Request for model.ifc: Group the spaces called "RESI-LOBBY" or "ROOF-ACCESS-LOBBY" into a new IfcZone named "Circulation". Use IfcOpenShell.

First a look at what the model holds.

```python
import ifcopenshell

model = ifcopenshell.open("model.ifc")
print(model.schema)
seen = {}
for space in model.by_type("IfcSpace"):
    seen[space.Name] = seen.get(space.Name, 0) + 1
for name, count in sorted(seen.items(), key=str):
    print(count, "x", name)
print("zones:", [z.Name for z in model.by_type("IfcZone")][:20])
```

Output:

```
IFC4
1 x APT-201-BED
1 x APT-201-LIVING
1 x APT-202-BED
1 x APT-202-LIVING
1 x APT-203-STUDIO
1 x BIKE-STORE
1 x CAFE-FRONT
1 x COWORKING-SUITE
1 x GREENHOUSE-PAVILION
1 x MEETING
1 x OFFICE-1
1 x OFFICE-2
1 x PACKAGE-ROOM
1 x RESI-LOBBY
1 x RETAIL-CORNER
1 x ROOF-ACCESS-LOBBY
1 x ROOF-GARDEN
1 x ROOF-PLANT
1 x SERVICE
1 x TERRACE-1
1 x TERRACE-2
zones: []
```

```python
import ifcopenshell
import ifcopenshell.api.group
import ifcopenshell.api.root

model = ifcopenshell.open("model.ifc")

names = {"RESI-LOBBY", "ROOF-ACCESS-LOBBY"}
spaces = [s for s in model.by_type("IfcSpace") if s.Name in names]

zone = ifcopenshell.api.root.create_entity(model, ifc_class="IfcZone", name="Circulation")
ifcopenshell.api.group.assign_group(model, products=spaces, group=zone)
print(len(spaces), "spaces in", zone.Name)

model.write("model_updated.ifc")
```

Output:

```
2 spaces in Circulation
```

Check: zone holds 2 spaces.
